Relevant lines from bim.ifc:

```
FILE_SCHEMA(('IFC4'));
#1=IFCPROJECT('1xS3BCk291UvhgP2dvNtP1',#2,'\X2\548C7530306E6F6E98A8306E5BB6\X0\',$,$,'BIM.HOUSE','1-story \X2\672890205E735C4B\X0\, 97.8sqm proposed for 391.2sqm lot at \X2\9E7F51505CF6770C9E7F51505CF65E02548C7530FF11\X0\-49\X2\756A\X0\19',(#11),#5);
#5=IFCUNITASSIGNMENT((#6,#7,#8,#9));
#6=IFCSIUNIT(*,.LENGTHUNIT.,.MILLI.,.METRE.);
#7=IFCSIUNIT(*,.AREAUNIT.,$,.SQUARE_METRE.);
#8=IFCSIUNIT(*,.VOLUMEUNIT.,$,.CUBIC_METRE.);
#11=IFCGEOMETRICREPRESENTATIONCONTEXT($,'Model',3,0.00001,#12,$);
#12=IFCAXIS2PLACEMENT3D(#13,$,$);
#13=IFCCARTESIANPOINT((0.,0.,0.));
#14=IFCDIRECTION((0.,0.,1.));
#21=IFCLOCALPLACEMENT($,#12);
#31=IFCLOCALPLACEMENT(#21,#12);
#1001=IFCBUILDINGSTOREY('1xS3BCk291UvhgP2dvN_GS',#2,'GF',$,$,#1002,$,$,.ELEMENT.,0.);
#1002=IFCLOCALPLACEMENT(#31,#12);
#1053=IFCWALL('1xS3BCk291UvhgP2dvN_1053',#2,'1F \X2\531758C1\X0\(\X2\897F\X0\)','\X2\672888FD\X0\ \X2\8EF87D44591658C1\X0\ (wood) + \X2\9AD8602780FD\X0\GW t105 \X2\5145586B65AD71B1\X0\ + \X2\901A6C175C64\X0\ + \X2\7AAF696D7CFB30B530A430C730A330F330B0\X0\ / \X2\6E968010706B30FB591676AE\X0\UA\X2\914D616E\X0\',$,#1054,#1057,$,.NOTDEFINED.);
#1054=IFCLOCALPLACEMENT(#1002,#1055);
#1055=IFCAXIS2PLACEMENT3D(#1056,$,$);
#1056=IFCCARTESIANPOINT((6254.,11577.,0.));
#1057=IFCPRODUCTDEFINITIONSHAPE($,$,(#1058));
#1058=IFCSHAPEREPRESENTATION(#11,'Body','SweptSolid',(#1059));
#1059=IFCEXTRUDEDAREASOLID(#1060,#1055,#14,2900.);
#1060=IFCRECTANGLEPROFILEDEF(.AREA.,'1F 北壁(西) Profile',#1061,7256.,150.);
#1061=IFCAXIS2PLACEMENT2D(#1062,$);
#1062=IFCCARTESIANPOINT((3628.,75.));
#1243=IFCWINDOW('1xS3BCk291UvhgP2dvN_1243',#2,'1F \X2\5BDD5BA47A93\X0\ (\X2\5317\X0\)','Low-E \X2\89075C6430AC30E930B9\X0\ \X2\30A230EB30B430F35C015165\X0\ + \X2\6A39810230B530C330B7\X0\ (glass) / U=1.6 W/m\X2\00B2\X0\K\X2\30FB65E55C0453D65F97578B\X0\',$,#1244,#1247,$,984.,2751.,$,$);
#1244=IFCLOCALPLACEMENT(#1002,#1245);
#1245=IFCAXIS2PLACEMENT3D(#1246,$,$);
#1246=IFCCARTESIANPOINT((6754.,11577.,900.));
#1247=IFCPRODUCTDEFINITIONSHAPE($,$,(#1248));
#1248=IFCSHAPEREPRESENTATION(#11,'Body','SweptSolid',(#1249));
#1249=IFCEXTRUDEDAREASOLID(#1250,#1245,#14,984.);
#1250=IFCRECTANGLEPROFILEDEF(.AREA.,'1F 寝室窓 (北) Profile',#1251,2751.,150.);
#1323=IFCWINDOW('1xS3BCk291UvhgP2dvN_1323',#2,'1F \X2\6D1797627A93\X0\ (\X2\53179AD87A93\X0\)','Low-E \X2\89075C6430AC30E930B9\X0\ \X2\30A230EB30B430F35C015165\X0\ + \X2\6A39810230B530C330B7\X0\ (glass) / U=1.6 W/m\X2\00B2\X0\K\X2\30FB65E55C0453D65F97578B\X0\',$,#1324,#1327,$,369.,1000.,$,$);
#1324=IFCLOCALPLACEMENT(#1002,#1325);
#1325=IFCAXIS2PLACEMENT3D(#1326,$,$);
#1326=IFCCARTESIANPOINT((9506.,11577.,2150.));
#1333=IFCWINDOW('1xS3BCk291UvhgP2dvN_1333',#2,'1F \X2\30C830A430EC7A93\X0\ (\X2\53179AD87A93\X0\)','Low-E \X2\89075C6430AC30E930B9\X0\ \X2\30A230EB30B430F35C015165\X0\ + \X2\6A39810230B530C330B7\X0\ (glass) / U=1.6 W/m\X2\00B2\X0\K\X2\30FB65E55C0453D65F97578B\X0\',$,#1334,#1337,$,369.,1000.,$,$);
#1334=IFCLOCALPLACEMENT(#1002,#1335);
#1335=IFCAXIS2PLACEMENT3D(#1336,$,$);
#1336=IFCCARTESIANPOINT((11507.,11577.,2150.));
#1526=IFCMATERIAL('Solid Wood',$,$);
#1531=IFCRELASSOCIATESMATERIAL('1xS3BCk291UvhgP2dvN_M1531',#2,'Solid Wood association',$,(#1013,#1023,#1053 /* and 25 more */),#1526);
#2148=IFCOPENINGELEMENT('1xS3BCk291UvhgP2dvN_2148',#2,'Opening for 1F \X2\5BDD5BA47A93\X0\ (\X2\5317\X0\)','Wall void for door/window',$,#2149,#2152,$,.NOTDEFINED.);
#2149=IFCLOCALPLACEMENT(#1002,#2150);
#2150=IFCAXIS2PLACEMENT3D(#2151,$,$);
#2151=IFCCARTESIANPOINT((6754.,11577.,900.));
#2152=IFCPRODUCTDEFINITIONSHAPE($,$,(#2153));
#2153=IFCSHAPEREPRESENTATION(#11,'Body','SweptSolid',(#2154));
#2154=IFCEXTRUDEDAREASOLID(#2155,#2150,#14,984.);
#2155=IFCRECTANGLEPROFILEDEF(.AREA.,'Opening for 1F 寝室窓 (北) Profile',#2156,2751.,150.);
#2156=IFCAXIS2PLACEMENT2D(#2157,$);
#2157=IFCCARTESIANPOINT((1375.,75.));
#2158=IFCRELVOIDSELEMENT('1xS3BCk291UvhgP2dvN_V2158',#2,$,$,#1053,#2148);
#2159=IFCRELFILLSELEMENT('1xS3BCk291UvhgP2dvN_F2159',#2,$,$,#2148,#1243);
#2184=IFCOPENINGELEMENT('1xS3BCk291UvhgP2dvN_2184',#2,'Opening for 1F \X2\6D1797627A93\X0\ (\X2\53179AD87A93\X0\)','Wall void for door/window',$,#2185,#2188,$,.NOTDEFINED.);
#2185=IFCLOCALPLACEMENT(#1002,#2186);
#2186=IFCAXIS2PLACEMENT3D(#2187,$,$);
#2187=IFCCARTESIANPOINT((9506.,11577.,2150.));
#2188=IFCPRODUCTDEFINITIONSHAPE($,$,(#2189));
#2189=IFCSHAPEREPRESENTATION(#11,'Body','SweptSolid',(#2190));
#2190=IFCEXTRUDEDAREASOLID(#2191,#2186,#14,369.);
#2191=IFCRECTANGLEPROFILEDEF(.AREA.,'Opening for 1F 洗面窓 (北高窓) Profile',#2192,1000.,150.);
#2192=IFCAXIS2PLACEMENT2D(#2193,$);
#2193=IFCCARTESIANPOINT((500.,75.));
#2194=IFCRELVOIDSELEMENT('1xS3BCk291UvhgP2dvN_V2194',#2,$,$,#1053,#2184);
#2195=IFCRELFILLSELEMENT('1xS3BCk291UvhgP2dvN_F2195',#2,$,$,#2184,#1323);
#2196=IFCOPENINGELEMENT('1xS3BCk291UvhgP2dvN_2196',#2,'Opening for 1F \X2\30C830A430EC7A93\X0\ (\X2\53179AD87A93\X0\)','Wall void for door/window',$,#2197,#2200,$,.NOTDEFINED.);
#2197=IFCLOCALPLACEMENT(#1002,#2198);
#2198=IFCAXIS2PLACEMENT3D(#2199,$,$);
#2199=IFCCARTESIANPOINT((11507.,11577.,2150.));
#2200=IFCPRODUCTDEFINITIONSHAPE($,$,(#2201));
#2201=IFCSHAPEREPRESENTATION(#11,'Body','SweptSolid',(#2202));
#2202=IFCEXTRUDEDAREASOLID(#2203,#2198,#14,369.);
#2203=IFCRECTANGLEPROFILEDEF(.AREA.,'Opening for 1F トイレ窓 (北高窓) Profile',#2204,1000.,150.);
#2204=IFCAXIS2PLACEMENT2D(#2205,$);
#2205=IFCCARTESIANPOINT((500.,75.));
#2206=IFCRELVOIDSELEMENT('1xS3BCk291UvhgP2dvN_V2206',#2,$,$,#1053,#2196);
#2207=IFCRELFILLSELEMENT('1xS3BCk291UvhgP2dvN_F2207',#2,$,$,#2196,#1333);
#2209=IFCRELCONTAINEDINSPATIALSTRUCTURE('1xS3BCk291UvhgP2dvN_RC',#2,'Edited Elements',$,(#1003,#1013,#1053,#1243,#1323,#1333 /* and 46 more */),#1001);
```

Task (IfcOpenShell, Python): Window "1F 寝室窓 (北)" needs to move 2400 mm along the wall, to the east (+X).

```python
import ifcopenshell
import ifcopenshell.api.geometry
import ifcopenshell.util.placement

model = ifcopenshell.open("bim.ifc")

window = model.by_guid("1xS3BCk291UvhgP2dvN_1243")
opening = window.FillsVoids[0].RelatingOpeningElement
wall = opening.VoidsElements[0].RelatingBuildingElement

wall_matrix = ifcopenshell.util.placement.get_local_placement(wall.ObjectPlacement)
shift = wall_matrix[:3, 0] * 2400.0
before = ifcopenshell.util.placement.get_local_placement(window.ObjectPlacement)[:3, 3].copy()

# The window is not placed relative to its opening, so move both.
for product in (opening, window):
    matrix = ifcopenshell.util.placement.get_local_placement(product.ObjectPlacement)
    matrix[:3, 3] += shift
    ifcopenshell.api.geometry.edit_object_placement(model, product=product, matrix=matrix, is_si=False)

after = ifcopenshell.util.placement.get_local_placement(window.ObjectPlacement)[:3, 3]
print("window moved by", (after - before).round(3) + 0.0)

model.write("bim_edited.ifc")
```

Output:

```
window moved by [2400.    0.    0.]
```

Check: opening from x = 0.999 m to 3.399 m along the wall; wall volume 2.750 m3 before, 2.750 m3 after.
